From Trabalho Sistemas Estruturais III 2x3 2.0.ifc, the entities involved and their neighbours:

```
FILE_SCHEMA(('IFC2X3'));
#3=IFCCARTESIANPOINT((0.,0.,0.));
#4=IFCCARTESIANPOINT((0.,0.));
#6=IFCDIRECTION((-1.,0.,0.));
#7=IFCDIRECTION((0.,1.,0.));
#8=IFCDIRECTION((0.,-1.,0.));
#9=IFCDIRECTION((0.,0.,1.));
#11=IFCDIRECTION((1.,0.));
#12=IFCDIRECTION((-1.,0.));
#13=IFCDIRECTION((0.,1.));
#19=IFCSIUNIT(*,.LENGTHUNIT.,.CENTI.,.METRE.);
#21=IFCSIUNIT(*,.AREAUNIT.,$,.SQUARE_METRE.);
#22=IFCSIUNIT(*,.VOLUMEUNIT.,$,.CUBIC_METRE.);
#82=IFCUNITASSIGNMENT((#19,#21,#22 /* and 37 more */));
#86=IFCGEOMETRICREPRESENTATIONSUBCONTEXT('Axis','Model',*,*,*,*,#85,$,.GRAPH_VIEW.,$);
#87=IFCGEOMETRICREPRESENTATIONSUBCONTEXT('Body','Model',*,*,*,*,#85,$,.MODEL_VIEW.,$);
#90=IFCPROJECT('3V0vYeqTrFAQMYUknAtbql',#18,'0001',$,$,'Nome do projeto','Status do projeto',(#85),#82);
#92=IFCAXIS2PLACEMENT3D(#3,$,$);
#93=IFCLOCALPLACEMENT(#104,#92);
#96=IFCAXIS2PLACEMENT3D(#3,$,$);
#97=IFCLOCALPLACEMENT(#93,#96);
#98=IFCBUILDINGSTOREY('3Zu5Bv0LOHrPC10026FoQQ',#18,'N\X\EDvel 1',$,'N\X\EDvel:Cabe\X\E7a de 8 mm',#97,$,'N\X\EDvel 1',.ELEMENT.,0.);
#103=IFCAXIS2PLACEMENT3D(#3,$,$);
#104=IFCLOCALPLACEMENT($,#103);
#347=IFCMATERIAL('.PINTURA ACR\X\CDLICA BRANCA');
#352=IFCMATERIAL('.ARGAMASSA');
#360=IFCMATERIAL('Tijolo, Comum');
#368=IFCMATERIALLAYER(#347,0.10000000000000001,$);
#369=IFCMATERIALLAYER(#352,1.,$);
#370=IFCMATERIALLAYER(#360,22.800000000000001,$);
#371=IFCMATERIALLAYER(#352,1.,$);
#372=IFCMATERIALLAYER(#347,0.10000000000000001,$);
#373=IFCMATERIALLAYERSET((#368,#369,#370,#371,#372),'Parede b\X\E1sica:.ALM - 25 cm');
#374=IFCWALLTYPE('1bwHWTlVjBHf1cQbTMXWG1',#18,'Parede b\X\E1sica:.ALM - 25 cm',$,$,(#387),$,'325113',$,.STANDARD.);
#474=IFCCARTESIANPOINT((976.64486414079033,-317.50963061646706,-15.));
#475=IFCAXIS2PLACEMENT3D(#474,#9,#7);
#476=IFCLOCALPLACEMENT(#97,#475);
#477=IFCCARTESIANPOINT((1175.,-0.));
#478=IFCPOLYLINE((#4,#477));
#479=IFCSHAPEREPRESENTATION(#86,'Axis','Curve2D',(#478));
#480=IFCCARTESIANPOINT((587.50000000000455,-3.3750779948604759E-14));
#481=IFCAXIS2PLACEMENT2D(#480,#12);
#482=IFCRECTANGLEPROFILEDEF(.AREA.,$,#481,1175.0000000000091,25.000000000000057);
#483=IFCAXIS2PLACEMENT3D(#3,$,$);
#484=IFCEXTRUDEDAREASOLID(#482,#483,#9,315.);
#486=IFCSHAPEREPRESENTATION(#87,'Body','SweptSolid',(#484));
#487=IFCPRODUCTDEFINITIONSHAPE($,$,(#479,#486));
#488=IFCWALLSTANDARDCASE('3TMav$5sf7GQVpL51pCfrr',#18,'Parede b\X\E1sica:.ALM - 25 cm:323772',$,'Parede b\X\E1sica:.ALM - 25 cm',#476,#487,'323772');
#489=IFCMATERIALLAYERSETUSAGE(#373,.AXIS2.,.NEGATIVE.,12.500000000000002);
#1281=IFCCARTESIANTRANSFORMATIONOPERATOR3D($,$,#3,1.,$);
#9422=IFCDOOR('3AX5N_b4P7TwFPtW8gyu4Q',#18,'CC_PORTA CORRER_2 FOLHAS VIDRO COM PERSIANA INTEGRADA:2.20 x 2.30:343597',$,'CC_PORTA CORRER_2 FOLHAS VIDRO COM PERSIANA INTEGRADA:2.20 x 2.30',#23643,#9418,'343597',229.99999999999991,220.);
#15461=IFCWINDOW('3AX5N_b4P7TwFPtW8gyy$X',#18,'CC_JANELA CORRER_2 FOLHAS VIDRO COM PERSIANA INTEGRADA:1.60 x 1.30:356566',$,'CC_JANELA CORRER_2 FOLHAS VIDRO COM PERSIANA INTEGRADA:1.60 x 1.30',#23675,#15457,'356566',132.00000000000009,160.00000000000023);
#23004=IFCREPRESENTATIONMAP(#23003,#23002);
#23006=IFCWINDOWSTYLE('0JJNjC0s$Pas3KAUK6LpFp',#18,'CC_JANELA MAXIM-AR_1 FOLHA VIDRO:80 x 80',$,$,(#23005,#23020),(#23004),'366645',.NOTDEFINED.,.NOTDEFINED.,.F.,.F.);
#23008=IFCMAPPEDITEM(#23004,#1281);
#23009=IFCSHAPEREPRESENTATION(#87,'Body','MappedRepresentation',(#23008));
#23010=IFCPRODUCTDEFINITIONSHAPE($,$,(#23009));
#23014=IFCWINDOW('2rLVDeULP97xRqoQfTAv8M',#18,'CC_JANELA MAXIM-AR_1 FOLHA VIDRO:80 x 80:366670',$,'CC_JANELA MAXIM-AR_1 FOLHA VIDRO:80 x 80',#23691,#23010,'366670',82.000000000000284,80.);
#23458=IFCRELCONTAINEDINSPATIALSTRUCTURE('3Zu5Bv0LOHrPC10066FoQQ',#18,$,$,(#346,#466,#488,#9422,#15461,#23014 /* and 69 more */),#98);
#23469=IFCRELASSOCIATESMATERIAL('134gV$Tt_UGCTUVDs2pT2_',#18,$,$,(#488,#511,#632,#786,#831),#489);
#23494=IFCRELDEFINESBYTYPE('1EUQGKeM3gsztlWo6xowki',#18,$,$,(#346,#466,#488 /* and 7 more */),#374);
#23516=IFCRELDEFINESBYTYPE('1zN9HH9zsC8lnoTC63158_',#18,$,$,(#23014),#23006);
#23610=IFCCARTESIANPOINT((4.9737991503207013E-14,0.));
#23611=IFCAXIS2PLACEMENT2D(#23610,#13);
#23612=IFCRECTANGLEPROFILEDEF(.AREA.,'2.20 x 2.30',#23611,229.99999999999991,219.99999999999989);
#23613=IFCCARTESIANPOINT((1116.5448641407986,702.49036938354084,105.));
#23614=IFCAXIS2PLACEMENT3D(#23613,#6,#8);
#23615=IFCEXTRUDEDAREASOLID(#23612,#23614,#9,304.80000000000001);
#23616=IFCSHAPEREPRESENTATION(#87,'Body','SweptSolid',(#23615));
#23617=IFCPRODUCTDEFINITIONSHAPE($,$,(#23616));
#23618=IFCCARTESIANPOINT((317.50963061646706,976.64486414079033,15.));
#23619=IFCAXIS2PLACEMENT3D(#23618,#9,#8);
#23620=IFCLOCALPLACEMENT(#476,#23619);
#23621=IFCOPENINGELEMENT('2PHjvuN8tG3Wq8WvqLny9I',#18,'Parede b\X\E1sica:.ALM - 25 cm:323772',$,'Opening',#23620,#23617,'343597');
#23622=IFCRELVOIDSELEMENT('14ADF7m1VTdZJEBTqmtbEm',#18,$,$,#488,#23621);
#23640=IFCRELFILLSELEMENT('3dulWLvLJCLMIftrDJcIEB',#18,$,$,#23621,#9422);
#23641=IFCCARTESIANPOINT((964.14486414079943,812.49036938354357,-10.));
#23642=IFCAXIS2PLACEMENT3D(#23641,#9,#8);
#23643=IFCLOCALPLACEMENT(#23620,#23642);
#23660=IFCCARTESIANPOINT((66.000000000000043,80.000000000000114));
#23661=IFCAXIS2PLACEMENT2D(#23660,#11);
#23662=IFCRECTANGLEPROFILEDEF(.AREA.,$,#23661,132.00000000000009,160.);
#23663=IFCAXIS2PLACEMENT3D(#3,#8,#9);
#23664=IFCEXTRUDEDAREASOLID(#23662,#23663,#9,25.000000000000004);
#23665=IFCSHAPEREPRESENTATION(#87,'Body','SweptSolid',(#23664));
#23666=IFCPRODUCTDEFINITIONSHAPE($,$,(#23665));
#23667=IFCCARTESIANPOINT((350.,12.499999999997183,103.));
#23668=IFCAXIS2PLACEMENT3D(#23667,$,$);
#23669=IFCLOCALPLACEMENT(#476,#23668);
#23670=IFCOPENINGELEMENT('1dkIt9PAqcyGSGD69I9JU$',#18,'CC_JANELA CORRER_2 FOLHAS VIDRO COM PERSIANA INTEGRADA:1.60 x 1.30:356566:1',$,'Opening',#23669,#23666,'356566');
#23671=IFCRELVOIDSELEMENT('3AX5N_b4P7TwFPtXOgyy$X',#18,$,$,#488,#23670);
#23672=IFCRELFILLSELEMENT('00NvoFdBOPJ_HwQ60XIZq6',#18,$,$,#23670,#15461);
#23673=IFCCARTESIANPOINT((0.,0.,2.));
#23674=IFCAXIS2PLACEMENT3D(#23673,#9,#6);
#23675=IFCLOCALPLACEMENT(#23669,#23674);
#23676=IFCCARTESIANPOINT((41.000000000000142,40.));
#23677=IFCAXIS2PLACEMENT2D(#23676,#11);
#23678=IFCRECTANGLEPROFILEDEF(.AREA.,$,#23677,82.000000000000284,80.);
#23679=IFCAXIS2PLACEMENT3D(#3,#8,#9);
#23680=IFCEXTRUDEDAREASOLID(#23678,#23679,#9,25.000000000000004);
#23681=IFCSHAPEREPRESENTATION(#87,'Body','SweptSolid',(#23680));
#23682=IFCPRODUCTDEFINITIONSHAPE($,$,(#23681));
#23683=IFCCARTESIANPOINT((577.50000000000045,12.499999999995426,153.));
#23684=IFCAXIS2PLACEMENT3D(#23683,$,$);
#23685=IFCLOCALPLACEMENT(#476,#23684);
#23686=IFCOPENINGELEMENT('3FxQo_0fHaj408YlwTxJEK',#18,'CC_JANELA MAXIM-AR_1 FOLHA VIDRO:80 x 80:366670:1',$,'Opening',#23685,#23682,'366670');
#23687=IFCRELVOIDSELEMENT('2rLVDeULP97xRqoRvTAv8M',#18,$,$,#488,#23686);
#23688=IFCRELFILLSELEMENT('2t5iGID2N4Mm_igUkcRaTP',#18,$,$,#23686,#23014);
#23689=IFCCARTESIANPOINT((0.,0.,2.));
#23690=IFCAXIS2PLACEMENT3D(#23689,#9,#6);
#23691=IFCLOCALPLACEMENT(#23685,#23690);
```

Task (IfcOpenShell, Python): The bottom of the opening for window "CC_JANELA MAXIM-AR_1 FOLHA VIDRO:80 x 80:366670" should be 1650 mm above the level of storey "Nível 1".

```python
import numpy as np
import ifcopenshell
import ifcopenshell.api.geometry
import ifcopenshell.geom
import ifcopenshell.util.element
import ifcopenshell.util.placement
import ifcopenshell.util.shape
import ifcopenshell.util.unit

model = ifcopenshell.open("Trabalho Sistemas Estruturais III 2x3 2.0.ifc")
unit_scale = ifcopenshell.util.unit.calculate_unit_scale(model)

window = model.by_id(23014)
opening = window.FillsVoids[0].RelatingOpeningElement
storey = ifcopenshell.util.element.get_container(window, ifc_class="IfcBuildingStorey")
level = ifcopenshell.util.placement.get_local_placement(storey.ObjectPlacement)[2, 3]

# The opening's origin need not be at the sill, so measure its lowest point.
shape = ifcopenshell.geom.create_shape(ifcopenshell.geom.settings(), opening)
bottom = ifcopenshell.util.shape.get_shape_bottom_elevation(shape, shape.geometry) / unit_scale
dz = level + 1.65 / unit_scale - bottom

shift = np.array([0.0, 0.0, dz])
# The window is placed relative to its opening, so it follows when the opening moves.
matrix = ifcopenshell.util.placement.get_local_placement(opening.ObjectPlacement)
matrix[:3, 3] += shift
ifcopenshell.api.geometry.edit_object_placement(
    model, product=opening, matrix=matrix, is_si=False, should_transform_children=True
)

print(f"moved by {dz * unit_scale:+.3f} m")

model.write("Trabalho Sistemas Estruturais III 2x3 2.0_rev.ifc")
```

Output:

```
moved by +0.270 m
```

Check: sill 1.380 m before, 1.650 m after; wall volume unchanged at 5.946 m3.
